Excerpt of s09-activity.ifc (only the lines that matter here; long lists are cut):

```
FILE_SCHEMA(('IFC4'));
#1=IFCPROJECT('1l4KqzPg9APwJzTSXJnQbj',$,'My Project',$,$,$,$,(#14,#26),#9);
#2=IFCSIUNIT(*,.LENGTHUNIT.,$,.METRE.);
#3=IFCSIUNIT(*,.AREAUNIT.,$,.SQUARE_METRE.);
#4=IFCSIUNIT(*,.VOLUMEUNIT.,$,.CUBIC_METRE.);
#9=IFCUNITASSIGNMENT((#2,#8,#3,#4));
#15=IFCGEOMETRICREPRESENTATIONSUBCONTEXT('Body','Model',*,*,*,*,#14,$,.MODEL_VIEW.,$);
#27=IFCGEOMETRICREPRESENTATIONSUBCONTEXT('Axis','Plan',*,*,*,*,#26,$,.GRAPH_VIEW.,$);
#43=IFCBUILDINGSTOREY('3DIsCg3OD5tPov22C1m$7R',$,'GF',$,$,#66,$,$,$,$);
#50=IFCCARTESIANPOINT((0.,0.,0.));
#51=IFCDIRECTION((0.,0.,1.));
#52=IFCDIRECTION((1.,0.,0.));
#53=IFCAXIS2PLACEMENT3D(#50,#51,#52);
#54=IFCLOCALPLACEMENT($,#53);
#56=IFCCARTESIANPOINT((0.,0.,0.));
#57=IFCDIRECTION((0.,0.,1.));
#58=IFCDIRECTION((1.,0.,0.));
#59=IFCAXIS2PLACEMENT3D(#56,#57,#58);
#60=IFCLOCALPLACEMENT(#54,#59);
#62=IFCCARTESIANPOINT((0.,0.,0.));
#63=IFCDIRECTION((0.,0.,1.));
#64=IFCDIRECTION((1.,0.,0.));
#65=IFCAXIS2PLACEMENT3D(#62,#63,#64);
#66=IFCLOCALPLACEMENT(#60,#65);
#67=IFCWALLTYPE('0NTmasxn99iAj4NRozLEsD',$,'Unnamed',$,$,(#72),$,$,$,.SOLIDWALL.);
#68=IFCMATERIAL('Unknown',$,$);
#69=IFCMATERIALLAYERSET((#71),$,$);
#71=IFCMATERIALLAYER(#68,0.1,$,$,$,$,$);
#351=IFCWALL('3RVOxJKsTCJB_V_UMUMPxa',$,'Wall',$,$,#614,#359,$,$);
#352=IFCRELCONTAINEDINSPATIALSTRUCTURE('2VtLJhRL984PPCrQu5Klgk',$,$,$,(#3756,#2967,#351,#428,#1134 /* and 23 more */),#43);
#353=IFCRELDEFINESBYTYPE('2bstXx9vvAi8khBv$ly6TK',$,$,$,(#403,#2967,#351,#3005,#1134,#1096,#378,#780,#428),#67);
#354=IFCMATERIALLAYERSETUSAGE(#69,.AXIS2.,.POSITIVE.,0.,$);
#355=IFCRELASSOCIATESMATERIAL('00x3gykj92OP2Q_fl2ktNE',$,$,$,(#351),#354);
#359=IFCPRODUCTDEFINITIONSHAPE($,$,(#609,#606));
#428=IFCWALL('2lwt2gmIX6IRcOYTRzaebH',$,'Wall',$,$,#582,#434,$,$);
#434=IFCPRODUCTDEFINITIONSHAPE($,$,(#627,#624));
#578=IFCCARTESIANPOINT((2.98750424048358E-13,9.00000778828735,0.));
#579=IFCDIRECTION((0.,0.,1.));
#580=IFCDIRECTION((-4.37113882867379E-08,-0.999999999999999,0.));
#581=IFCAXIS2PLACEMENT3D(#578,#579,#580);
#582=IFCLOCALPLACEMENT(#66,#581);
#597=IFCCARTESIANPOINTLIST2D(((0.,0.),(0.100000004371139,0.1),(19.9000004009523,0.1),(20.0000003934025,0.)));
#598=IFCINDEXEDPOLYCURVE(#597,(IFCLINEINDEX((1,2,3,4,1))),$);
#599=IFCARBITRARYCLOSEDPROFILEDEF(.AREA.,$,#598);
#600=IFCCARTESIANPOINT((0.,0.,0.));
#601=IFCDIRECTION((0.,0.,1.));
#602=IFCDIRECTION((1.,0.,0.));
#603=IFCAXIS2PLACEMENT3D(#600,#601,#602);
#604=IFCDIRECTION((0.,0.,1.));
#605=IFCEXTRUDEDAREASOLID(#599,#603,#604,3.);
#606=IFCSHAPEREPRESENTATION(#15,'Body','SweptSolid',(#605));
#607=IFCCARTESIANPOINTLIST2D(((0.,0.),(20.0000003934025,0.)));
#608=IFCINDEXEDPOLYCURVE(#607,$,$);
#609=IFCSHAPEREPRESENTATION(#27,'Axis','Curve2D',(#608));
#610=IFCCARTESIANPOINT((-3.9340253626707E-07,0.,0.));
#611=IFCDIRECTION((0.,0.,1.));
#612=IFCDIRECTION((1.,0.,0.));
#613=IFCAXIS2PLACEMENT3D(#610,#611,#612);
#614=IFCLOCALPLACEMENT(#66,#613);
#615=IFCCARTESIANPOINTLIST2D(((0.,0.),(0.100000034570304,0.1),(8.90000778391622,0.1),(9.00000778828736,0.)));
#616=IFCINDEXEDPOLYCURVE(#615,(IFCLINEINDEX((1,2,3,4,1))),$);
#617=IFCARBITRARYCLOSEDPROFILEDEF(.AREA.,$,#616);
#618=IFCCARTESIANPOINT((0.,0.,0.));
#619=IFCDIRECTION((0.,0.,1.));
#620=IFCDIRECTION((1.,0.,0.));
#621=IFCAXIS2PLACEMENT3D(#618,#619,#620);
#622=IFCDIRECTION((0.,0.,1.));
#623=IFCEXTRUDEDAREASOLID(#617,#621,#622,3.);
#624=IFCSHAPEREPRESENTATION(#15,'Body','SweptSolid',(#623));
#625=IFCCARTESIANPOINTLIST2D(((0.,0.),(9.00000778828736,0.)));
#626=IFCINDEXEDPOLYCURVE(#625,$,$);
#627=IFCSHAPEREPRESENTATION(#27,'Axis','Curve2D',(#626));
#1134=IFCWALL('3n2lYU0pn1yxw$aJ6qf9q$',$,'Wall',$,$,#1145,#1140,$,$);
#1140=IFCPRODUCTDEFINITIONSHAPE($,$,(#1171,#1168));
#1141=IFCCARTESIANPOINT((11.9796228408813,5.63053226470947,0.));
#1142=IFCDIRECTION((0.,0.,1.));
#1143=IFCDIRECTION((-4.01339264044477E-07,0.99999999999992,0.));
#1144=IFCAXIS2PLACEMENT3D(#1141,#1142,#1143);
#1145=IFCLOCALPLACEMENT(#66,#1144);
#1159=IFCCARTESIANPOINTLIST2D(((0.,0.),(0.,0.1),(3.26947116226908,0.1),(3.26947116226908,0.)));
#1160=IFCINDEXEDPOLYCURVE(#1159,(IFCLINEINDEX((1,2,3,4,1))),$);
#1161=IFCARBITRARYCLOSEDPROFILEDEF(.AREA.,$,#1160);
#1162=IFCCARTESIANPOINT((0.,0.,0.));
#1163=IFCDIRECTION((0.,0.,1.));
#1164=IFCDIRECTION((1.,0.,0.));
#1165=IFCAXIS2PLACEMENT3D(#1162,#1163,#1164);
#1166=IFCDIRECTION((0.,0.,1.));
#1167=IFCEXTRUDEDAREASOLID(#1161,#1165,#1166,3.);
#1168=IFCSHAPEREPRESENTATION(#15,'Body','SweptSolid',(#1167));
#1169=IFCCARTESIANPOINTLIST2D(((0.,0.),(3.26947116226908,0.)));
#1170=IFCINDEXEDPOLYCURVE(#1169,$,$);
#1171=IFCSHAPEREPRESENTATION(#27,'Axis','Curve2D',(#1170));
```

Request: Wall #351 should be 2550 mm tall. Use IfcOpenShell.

```python
import ifcopenshell
import ifcopenshell.geom
import ifcopenshell.util.representation
import ifcopenshell.util.shape

model = ifcopenshell.open("s09-activity.ifc")
settings = ifcopenshell.geom.settings()


def volume(element):
    """Net volume in cubic metres, openings subtracted."""
    shape = ifcopenshell.geom.create_shape(settings, element)
    return ifcopenshell.util.shape.get_volume(shape.geometry)


wall = model.by_id(351)
before = volume(wall)

body = ifcopenshell.util.representation.get_representation(wall, "Model", "Body")
solid = body.Items[0]
old_height = solid.Depth
solid.Depth = 2.55
after = volume(wall)

print(f"height {old_height:g} -> {solid.Depth:g}, volume {before:.3f} -> {after:.3f} m3")

model.write("s09-activity-out.ifc")
```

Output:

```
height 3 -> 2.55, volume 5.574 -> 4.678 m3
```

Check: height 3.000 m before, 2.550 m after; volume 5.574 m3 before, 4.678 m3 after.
